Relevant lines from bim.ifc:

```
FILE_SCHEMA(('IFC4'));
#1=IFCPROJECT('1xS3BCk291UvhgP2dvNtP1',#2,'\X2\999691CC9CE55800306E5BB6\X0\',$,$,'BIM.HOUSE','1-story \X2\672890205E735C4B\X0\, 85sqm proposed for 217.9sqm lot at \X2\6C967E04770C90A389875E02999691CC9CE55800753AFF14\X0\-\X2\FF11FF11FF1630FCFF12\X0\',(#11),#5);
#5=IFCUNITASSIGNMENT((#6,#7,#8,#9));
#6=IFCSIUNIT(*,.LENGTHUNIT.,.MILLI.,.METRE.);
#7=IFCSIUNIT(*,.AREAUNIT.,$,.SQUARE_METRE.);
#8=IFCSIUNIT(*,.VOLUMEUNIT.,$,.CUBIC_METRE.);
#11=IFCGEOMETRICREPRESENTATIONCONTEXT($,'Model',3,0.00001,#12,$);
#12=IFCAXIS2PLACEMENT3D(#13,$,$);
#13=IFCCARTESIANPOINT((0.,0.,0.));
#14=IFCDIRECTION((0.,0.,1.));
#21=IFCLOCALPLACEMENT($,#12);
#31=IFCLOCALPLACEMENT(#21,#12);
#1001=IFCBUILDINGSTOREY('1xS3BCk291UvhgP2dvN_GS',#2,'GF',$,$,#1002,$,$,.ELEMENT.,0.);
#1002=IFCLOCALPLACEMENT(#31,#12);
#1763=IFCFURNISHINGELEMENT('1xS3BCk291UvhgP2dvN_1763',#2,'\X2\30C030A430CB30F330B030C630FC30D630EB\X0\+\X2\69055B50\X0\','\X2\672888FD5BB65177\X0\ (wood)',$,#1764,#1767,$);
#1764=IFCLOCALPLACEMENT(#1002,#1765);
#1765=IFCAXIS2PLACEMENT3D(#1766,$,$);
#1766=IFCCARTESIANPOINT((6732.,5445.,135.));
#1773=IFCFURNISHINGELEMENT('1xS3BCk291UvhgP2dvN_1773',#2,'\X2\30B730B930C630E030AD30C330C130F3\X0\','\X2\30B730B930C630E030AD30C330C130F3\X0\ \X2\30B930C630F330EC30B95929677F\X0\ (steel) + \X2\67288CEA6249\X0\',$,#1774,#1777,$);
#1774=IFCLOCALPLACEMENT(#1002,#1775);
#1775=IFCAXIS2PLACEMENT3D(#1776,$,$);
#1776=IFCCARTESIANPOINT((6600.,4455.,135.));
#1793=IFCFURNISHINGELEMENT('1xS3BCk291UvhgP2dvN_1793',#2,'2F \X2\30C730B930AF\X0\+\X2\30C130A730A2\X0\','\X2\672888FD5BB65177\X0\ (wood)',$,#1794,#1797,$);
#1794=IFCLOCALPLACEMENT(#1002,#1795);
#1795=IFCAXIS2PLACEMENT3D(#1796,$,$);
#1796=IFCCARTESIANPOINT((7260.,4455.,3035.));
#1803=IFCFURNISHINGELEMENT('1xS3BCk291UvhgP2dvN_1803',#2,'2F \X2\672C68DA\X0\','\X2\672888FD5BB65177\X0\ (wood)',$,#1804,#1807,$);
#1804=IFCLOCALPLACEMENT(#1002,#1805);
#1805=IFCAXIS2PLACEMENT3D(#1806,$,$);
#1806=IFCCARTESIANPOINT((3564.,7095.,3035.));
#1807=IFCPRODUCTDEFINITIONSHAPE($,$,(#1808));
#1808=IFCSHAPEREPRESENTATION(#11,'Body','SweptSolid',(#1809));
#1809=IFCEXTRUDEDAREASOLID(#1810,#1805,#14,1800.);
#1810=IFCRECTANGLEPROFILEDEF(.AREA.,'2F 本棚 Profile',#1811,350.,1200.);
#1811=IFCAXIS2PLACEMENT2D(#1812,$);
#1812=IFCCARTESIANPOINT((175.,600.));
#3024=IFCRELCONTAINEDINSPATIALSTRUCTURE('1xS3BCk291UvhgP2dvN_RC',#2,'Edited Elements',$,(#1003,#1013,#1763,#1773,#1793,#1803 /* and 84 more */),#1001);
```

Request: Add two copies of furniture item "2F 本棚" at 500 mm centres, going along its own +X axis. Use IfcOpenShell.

```python
import ifcopenshell
import ifcopenshell.api.geometry
import ifcopenshell.api.root
import ifcopenshell.util.element
import ifcopenshell.util.placement

model = ifcopenshell.open("bim.ifc")


def reuse_history(source, copy):
    """copy_class also copies each property set's owner history, people and application; keep the originals."""
    for rel in copy.IsDefinedBy:
        if rel.is_a("IfcRelDefinesByProperties") and (history := rel.RelatingPropertyDefinition.OwnerHistory):
            rel.RelatingPropertyDefinition.OwnerHistory = source.OwnerHistory
            ifcopenshell.util.element.remove_deep2(model, history)


source = model.by_guid("1xS3BCk291UvhgP2dvN_1803")
base = ifcopenshell.util.placement.get_local_placement(source.ObjectPlacement)
step = base[:3, 0] * 500.0

for i in range(1, 3):
    copy = ifcopenshell.api.root.copy_class(model, product=source)
    copy.Representation = ifcopenshell.util.element.copy_deep(
        model, source.Representation, exclude=["IfcGeometricRepresentationContext", "IfcRepresentationMap"]
    )
    reuse_history(source, copy)
    matrix = base.copy()
    matrix[:3, 3] += i * step
    print("added at", matrix[:3, 3].round(3) + 0.0)
    ifcopenshell.api.geometry.edit_object_placement(model, product=copy, matrix=matrix, is_si=False)

model.write("bim_v2.ifc")
```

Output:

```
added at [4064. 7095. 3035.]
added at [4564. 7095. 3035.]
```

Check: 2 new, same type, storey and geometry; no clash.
